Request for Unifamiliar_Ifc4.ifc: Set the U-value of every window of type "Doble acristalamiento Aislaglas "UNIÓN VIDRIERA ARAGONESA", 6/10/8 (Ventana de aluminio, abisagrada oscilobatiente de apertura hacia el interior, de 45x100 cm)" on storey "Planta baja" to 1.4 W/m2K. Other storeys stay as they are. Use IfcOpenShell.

First a look at what the model holds.

```python
import ifcopenshell
import ifcopenshell.util.element

model = ifcopenshell.open("Unifamiliar_Ifc4.ifc")
print(model.schema)
storey = next(s for s in model.by_type("IfcBuildingStorey") if s.Name == "Planta baja")
windows = [e for e in ifcopenshell.util.element.get_decomposition(storey) if e.is_a("IfcWindow")]
seen = {}
for e in windows:
    element_type = ifcopenshell.util.element.get_type(e)
    key = (element_type.Name if element_type != e and element_type else None, ifcopenshell.util.element.get_pset(e, "Pset_WindowCommon", "ThermalTransmittance"))
    seen[key] = seen.get(key, 0) + 1
for (name, value), count in sorted(seen.items(), key=str):
    print(count, "x", name, "|", value)
```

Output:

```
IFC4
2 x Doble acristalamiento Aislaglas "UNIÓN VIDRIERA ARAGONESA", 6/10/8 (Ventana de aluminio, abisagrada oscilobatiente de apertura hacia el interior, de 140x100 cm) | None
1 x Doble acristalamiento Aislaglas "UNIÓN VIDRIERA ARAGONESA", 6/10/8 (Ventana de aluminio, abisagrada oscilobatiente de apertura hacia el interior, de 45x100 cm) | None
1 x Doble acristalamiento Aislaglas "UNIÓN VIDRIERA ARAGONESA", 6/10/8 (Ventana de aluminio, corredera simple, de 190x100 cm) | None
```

```python
import ifcopenshell
import ifcopenshell.api.pset
import ifcopenshell.util.element

model = ifcopenshell.open("Unifamiliar_Ifc4.ifc")

storey = next(s for s in model.by_type("IfcBuildingStorey") if s.Name == "Planta baja")
windows = [e for e in ifcopenshell.util.element.get_decomposition(storey) if e.is_a("IfcWindow")]

count = 0
for e in windows:
    element_type = ifcopenshell.util.element.get_type(e)
    if element_type in (None, e) or element_type.Name != 'Doble acristalamiento Aislaglas "UNIÓN VIDRIERA ARAGONESA", 6/10/8 (Ventana de aluminio, abisagrada oscilobatiente de apertura hacia el interior, de 45x100 cm)':
        continue
    # add_pset returns the element's existing set when there is one.
    pset = ifcopenshell.api.pset.add_pset(model, product=e, name="Pset_WindowCommon")
    ifcopenshell.api.pset.edit_pset(model, pset=pset, properties={"ThermalTransmittance": 1.4})
    count += 1

print(count, "windows updated")

model.write("Unifamiliar_Ifc4_rev.ifc")
```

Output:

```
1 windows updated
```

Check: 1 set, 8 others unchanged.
